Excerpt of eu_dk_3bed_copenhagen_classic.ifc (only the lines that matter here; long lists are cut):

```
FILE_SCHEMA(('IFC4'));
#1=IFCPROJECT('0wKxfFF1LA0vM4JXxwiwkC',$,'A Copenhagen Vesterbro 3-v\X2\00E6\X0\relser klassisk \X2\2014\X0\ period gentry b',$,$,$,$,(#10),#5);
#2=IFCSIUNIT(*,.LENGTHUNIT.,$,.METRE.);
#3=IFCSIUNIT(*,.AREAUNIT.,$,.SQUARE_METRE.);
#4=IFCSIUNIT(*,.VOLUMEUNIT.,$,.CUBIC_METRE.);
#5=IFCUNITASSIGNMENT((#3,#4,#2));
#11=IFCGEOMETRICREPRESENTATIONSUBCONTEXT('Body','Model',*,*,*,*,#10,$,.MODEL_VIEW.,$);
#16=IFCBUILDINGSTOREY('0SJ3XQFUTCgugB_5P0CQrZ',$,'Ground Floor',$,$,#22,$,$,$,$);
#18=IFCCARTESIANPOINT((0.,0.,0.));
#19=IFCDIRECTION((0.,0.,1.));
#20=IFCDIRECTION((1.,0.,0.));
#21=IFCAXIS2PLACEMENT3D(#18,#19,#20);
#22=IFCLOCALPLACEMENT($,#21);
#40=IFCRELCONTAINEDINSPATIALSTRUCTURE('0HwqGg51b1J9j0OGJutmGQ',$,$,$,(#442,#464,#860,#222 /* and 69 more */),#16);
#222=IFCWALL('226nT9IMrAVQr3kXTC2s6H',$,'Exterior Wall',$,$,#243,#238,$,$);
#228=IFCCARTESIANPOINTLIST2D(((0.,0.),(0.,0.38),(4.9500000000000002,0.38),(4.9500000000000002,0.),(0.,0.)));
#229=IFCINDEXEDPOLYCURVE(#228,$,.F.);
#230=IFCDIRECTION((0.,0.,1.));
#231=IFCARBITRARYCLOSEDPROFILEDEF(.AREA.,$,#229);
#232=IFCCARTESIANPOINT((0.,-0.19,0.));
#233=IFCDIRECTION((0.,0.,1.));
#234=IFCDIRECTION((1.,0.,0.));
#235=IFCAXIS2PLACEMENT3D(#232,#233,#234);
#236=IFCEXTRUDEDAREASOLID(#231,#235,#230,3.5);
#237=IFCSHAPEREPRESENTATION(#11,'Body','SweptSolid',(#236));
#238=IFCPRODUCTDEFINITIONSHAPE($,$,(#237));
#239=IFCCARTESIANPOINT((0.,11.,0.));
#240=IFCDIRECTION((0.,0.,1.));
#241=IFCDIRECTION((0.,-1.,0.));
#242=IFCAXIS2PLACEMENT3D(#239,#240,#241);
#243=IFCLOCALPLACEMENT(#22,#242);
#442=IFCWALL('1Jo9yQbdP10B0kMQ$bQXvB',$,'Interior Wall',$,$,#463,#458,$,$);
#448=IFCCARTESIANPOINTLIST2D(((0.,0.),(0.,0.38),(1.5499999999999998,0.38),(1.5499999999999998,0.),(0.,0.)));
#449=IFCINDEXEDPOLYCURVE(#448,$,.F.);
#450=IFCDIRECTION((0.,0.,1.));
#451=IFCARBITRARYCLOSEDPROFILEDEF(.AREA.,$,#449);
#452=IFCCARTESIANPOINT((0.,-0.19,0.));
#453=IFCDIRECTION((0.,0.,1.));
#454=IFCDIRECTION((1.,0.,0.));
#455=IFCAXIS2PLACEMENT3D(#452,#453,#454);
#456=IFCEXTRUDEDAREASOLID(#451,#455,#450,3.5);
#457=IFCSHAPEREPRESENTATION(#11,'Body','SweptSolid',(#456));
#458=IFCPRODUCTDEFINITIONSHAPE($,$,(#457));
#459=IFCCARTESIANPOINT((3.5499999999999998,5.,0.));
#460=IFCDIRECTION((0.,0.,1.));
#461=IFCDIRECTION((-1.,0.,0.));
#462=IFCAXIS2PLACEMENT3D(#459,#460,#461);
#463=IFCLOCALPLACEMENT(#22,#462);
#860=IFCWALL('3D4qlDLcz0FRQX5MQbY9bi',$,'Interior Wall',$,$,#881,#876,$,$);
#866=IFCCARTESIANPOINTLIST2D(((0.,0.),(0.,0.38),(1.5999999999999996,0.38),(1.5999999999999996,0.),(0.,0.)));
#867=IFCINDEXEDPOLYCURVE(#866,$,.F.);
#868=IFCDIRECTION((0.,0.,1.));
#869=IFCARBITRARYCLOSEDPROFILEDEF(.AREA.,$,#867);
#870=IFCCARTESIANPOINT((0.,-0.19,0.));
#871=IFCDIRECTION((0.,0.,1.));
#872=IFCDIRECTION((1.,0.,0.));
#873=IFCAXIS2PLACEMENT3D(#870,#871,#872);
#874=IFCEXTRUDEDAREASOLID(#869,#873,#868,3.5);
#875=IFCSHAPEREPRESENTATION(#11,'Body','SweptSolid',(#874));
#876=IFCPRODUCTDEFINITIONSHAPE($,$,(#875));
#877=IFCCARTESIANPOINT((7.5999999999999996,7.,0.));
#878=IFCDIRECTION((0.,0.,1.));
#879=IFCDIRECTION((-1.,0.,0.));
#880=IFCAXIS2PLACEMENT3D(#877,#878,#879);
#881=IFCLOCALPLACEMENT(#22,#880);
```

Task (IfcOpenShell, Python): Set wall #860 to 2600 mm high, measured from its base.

```python
import ifcopenshell
import ifcopenshell.geom
import ifcopenshell.util.representation
import ifcopenshell.util.shape
import ifcopenshell.util.unit

model = ifcopenshell.open("eu_dk_3bed_copenhagen_classic.ifc")
unit_scale = ifcopenshell.util.unit.calculate_unit_scale(model)
settings = ifcopenshell.geom.settings()


def volume(element):
    """Net volume in cubic metres, openings subtracted."""
    shape = ifcopenshell.geom.create_shape(settings, element)
    return ifcopenshell.util.shape.get_volume(shape.geometry)


wall = model.by_id(860)
before = volume(wall)

body = ifcopenshell.util.representation.get_representation(wall, "Model", "Body")
solid = body.Items[0]
old_height = solid.Depth
solid.Depth = 2.6 / unit_scale
after = volume(wall)

print(f"height {old_height:g} -> {solid.Depth:g}, volume {before:.3f} -> {after:.3f} m3")

model.write("eu_dk_3bed_copenhagen_classic_v2.ifc")
```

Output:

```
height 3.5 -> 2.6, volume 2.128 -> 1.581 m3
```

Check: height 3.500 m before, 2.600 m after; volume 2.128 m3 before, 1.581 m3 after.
